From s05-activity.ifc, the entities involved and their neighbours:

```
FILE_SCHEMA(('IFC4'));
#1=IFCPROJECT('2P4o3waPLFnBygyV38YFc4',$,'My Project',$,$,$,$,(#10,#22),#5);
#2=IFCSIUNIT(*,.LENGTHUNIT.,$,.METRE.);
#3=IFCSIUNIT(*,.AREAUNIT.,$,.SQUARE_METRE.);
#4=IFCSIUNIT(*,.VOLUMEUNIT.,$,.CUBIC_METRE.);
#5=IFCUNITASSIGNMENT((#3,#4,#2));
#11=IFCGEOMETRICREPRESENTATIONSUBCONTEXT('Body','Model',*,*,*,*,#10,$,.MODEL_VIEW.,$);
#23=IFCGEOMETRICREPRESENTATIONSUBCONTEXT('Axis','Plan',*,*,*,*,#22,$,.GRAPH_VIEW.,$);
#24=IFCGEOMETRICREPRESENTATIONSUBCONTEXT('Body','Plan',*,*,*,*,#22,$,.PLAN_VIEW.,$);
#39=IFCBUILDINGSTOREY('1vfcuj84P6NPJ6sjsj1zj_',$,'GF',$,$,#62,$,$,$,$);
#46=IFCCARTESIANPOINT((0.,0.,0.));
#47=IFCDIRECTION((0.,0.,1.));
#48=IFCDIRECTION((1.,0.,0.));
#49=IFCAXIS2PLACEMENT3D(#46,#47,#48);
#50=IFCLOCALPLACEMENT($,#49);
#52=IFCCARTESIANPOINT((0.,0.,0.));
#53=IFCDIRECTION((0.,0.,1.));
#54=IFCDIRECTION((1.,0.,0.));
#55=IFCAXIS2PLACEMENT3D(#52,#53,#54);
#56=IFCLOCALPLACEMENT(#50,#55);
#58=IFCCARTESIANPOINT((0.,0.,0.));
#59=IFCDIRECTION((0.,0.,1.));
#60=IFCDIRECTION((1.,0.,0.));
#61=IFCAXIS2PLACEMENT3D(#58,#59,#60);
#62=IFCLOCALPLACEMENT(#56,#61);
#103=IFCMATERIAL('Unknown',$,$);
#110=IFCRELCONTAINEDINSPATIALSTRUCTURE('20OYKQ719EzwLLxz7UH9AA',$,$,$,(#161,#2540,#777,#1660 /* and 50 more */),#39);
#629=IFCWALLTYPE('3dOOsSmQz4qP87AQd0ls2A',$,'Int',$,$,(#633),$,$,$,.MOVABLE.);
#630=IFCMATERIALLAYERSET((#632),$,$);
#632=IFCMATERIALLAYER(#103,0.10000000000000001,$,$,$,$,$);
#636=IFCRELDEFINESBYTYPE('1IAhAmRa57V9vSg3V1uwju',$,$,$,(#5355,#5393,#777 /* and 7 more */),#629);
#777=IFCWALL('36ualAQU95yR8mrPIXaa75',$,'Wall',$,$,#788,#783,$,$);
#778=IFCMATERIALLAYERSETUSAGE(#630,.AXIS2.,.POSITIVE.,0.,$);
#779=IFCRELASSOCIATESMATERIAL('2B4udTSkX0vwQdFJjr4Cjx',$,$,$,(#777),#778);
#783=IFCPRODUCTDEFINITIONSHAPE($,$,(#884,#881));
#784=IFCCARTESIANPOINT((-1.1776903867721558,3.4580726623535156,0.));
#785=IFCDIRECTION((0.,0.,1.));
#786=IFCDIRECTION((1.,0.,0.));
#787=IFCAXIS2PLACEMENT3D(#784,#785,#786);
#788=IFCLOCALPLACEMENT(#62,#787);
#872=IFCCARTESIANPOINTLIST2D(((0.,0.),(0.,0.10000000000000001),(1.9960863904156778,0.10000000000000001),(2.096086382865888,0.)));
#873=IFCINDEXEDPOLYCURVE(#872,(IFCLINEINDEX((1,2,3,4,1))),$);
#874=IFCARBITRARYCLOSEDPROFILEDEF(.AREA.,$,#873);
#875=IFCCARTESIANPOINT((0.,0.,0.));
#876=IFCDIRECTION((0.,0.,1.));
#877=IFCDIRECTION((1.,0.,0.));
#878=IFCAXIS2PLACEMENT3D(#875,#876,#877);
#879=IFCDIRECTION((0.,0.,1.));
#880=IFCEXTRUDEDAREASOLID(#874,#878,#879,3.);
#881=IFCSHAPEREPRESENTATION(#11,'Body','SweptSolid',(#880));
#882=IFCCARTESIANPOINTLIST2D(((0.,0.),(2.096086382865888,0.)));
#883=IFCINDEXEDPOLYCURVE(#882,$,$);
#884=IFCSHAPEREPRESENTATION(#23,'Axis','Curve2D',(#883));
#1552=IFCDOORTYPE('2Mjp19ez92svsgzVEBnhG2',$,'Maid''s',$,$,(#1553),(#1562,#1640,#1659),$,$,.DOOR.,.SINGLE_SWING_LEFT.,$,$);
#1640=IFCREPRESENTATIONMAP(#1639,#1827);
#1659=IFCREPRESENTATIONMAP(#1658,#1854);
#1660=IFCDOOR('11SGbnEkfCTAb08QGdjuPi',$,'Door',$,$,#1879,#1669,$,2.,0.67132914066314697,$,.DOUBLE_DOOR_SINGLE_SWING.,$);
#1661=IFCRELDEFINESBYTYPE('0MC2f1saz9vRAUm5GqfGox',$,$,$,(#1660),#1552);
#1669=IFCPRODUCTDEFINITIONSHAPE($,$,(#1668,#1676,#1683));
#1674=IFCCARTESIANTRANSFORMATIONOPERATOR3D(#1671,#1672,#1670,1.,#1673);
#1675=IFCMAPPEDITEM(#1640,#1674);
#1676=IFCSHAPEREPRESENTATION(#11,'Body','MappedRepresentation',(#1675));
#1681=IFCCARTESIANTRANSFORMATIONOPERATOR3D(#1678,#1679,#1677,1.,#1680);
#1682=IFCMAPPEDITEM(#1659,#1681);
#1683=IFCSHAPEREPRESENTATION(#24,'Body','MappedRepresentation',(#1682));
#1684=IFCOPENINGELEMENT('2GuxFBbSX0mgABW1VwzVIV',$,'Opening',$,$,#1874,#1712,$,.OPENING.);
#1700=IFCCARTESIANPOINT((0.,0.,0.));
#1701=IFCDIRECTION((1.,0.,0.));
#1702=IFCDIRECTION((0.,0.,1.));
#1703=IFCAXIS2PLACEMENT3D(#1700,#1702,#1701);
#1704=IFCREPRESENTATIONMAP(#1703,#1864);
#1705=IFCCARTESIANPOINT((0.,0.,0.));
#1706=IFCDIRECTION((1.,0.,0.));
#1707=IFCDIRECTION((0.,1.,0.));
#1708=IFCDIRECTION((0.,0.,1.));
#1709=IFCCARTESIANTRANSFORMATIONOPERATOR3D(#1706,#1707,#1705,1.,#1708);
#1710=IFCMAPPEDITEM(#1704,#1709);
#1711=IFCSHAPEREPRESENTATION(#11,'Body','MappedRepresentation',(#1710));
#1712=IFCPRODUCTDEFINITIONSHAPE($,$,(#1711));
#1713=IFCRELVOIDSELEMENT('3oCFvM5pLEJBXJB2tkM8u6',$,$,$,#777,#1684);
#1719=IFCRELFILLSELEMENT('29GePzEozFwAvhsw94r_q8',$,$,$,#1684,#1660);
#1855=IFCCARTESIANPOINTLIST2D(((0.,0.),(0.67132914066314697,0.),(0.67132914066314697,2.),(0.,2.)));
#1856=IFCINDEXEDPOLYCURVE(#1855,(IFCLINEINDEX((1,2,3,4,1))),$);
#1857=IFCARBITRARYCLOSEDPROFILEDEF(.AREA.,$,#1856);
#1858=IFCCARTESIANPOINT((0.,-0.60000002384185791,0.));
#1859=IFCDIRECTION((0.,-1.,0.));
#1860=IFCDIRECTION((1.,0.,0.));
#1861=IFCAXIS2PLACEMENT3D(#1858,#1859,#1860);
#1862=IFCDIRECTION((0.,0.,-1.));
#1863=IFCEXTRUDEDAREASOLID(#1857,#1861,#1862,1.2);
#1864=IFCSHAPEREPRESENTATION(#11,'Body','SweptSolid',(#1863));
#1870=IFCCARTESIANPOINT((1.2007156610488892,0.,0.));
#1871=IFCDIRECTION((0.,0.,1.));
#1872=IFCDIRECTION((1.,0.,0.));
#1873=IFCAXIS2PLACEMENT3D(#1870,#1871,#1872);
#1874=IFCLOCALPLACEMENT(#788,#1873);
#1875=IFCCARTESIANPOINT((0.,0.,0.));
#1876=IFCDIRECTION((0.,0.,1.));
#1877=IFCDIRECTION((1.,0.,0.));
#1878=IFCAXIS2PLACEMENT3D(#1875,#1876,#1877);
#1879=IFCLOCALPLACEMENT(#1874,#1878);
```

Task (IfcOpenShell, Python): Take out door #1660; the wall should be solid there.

```python
import ifcopenshell
import ifcopenshell.api.feature
import ifcopenshell.api.root
import ifcopenshell.geom
import ifcopenshell.util.shape

model = ifcopenshell.open("s05-activity.ifc")
settings = ifcopenshell.geom.settings()


def volume(element):
    """Net volume in cubic metres, openings subtracted."""
    shape = ifcopenshell.geom.create_shape(settings, element)
    return ifcopenshell.util.shape.get_volume(shape.geometry)


door = model.by_id(1660)
opening = door.FillsVoids[0].RelatingOpeningElement
wall = opening.VoidsElements[0].RelatingBuildingElement
before = volume(wall)

ifcopenshell.api.root.remove_product(model, product=door)
ifcopenshell.api.feature.remove_feature(model, feature=opening)

after = volume(wall)

print(f"wall volume {before:.3f} -> {after:.3f} m3")

model.write("s05-activity_rev.ifc")
```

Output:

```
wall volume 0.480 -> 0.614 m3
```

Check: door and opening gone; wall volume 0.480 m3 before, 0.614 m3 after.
